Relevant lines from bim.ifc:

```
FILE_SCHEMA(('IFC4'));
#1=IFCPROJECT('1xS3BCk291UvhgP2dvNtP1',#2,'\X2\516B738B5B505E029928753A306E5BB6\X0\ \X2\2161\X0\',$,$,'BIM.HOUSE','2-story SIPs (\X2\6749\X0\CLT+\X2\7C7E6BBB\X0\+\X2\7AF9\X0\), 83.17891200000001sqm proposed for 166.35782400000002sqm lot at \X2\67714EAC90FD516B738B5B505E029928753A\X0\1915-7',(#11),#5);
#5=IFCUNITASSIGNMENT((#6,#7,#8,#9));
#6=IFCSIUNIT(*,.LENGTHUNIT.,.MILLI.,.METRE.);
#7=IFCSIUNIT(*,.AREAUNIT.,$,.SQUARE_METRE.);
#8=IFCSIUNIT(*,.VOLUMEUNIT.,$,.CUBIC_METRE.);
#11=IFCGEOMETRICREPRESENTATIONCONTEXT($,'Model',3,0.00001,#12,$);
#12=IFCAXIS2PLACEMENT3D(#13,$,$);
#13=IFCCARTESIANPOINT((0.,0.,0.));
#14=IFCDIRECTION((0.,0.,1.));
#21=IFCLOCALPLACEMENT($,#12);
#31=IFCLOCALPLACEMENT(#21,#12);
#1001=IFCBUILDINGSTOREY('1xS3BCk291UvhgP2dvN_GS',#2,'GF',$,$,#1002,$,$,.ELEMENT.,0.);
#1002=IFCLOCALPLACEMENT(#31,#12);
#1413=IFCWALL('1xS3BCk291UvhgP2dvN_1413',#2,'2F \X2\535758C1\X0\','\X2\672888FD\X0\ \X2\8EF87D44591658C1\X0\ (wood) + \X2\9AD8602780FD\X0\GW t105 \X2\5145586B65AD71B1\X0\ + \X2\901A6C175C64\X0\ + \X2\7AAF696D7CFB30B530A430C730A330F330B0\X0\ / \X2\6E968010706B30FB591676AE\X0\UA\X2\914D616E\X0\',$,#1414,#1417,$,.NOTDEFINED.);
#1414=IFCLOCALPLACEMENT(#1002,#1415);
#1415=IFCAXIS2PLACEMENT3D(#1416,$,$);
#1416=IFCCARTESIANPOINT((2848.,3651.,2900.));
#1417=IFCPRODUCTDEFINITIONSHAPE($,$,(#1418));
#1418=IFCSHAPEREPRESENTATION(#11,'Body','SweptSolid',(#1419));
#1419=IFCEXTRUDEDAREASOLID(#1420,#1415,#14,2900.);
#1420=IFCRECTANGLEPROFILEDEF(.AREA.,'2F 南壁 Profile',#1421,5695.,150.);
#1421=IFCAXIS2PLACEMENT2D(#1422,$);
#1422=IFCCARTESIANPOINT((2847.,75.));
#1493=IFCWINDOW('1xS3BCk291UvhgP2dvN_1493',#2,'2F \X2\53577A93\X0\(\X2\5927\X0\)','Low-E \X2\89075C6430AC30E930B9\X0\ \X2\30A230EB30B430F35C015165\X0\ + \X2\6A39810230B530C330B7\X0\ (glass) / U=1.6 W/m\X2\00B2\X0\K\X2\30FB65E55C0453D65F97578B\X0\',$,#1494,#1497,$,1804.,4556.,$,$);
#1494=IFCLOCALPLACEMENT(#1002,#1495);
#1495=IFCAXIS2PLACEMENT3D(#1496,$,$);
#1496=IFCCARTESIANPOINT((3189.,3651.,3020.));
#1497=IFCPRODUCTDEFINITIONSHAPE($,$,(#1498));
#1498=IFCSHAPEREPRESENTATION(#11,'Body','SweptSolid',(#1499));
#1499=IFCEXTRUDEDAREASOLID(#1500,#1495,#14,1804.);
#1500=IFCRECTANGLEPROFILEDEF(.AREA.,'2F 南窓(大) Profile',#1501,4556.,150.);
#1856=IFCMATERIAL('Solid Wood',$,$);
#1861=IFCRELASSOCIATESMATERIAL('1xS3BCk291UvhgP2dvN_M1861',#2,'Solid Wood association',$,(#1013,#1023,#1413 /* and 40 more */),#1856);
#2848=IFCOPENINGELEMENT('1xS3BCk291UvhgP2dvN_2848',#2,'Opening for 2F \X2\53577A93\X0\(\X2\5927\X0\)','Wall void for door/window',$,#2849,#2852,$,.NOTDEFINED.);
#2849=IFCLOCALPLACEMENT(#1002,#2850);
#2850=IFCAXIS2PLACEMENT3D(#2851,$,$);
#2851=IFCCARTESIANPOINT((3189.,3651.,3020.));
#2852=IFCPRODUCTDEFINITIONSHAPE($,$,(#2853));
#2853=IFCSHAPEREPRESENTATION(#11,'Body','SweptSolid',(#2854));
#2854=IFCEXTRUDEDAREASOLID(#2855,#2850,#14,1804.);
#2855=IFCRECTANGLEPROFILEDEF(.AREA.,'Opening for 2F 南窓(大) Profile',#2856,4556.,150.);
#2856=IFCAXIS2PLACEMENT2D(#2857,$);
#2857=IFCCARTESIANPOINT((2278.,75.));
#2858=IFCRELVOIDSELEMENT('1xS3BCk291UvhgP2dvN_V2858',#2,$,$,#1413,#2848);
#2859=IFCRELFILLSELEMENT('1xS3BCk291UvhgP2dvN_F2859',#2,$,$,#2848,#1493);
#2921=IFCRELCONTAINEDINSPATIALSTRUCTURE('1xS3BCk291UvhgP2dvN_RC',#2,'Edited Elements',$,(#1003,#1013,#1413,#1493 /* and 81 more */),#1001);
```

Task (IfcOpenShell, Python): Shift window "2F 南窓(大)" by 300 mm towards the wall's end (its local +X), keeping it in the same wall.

```python
import ifcopenshell
import ifcopenshell.api.geometry
import ifcopenshell.util.placement

model = ifcopenshell.open("bim.ifc")

window = model.by_guid("1xS3BCk291UvhgP2dvN_1493")
opening = window.FillsVoids[0].RelatingOpeningElement
wall = opening.VoidsElements[0].RelatingBuildingElement

wall_matrix = ifcopenshell.util.placement.get_local_placement(wall.ObjectPlacement)
shift = wall_matrix[:3, 0] * 300.0
before = ifcopenshell.util.placement.get_local_placement(window.ObjectPlacement)[:3, 3].copy()

# The window is not placed relative to its opening, so move both.
for product in (opening, window):
    matrix = ifcopenshell.util.placement.get_local_placement(product.ObjectPlacement)
    matrix[:3, 3] += shift
    ifcopenshell.api.geometry.edit_object_placement(model, product=product, matrix=matrix, is_si=False)

after = ifcopenshell.util.placement.get_local_placement(window.ObjectPlacement)[:3, 3]
print("window moved by", (after - before).round(3) + 0.0)

model.write("bim_rev.ifc")
```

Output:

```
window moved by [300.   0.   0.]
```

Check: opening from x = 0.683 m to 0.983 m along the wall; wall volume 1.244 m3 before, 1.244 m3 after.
